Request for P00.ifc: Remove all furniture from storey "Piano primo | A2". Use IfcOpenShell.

First a look at what the model holds.

```python
import ifcopenshell
import ifcopenshell.util.element

model = ifcopenshell.open("P00.ifc")
print(model.schema)
storey = next(s for s in model.by_type("IfcBuildingStorey") if s.Name == "Piano primo | A2")
furniture = [e for e in ifcopenshell.util.element.get_decomposition(storey) if e.is_a("IfcFurnishingElement")]
seen = {}
for e in furniture:
    element_type = ifcopenshell.util.element.get_type(e)
    name = element_type.Name if element_type not in (None, e) else None
    seen[name] = seen.get(name, 0) + 1
for name, count in sorted(seen.items(), key=str):
    print(count, "x", name)
```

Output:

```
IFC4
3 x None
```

```python
import ifcopenshell
import ifcopenshell.api.root
import ifcopenshell.util.element

model = ifcopenshell.open("P00.ifc")

storey = next(s for s in model.by_type("IfcBuildingStorey") if s.Name == "Piano primo | A2")
furniture = [e for e in ifcopenshell.util.element.get_decomposition(storey) if e.is_a("IfcFurnishingElement")]

for e in furniture:
    ifcopenshell.api.root.remove_product(model, product=e)
print(len(furniture), "removed")

model.write("P00_updated.ifc")
```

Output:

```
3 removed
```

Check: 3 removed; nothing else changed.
